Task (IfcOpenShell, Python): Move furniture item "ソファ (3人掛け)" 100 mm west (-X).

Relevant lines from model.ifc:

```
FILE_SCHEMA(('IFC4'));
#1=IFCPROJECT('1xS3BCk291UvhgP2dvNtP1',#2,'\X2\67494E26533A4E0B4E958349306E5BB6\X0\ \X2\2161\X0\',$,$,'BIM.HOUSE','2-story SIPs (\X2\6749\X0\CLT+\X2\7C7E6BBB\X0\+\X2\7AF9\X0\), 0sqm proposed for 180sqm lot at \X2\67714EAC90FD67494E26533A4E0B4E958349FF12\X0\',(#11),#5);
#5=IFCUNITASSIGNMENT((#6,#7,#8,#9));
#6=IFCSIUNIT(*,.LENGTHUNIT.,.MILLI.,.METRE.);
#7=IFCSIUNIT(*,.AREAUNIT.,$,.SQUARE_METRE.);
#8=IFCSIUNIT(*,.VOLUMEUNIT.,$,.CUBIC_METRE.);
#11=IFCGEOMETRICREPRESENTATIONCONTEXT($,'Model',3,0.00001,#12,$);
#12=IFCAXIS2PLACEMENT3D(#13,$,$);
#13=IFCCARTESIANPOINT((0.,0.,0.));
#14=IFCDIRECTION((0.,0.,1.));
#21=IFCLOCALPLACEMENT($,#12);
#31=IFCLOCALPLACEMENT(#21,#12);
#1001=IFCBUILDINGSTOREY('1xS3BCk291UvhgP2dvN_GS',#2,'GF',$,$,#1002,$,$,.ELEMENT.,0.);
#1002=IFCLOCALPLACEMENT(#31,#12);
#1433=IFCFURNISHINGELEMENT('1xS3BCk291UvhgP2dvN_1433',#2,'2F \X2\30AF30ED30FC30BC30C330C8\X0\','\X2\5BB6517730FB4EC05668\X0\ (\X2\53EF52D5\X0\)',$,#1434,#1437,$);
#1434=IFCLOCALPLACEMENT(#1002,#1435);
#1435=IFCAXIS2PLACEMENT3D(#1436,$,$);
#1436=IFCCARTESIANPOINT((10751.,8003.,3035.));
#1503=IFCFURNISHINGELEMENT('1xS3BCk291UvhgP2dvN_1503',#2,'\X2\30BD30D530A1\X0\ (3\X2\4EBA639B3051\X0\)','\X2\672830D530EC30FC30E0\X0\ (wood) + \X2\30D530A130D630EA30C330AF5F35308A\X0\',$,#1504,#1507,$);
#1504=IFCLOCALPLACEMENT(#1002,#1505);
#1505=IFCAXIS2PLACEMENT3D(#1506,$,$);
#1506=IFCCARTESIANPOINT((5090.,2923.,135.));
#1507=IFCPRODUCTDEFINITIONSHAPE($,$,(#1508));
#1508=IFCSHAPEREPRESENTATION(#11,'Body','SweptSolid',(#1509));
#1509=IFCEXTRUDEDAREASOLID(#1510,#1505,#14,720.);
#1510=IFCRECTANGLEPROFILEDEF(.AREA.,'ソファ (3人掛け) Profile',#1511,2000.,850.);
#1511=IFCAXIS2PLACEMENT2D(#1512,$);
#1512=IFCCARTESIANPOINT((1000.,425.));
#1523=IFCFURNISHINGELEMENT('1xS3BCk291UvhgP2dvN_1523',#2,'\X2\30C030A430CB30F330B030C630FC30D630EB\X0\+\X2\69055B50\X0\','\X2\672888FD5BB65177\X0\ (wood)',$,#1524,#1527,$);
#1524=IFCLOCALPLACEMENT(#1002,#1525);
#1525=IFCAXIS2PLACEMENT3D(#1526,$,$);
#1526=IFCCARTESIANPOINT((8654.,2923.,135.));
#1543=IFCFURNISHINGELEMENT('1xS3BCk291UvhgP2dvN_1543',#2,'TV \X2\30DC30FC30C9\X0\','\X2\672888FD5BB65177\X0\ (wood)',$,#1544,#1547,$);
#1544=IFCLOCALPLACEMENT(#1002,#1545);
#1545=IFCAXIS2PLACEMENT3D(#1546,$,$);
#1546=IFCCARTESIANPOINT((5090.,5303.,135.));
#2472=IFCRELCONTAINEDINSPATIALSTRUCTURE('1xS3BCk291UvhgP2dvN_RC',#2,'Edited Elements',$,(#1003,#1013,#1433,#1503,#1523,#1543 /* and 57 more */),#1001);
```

```python
import ifcopenshell
import ifcopenshell.api.geometry
import ifcopenshell.util.placement

model = ifcopenshell.open("model.ifc")

item = model.by_id(1503)
matrix = ifcopenshell.util.placement.get_local_placement(item.ObjectPlacement)
matrix[0, 3] -= 100.0
ifcopenshell.api.geometry.edit_object_placement(model, product=item, matrix=matrix, is_si=False)

print(ifcopenshell.util.placement.get_local_placement(item.ObjectPlacement).round(3) + 0.0)

model.write("model_edited.ifc")
```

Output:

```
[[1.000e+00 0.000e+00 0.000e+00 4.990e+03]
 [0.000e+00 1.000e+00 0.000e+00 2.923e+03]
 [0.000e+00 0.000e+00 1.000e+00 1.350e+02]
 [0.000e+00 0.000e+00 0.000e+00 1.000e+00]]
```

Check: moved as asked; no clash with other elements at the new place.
